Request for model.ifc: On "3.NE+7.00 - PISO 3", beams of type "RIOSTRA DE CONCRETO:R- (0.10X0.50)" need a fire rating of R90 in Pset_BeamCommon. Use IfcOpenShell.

First a look at what the model holds.

```python
import ifcopenshell
import ifcopenshell.util.element

model = ifcopenshell.open("model.ifc")
print(model.schema)
storey = next(s for s in model.by_type("IfcBuildingStorey") if s.Name == "3.NE+7.00 - PISO 3")
beams = [e for e in ifcopenshell.util.element.get_decomposition(storey) if e.is_a("IfcBeam")]
seen = {}
for e in beams:
    element_type = ifcopenshell.util.element.get_type(e)
    key = (element_type.Name if element_type != e and element_type else None, ifcopenshell.util.element.get_pset(e, "Pset_BeamCommon", "FireRating"))
    seen[key] = seen.get(key, 0) + 1
for (name, value), count in sorted(seen.items(), key=str):
    print(count, "x", name, "|", value)
```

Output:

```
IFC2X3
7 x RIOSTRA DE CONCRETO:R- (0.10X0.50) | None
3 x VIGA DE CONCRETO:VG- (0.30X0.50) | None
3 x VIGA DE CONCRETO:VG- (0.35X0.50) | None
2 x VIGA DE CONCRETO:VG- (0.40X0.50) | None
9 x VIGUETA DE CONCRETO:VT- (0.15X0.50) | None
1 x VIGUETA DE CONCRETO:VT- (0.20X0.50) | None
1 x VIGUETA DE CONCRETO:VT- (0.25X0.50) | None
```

```python
import ifcopenshell
import ifcopenshell.api.pset
import ifcopenshell.util.element

model = ifcopenshell.open("model.ifc")

storey = next(s for s in model.by_type("IfcBuildingStorey") if s.Name == "3.NE+7.00 - PISO 3")
beams = [e for e in ifcopenshell.util.element.get_decomposition(storey) if e.is_a("IfcBeam")]

count = 0
for e in beams:
    element_type = ifcopenshell.util.element.get_type(e)
    if element_type in (None, e) or element_type.Name != "RIOSTRA DE CONCRETO:R- (0.10X0.50)":
        continue
    # add_pset returns the element's existing set when there is one.
    pset = ifcopenshell.api.pset.add_pset(model, product=e, name="Pset_BeamCommon")
    ifcopenshell.api.pset.edit_pset(model, pset=pset, properties={"FireRating": "R90"})
    count += 1

print(count, "beams updated")

model.write("model-out.ifc")
```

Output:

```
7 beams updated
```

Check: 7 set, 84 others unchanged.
